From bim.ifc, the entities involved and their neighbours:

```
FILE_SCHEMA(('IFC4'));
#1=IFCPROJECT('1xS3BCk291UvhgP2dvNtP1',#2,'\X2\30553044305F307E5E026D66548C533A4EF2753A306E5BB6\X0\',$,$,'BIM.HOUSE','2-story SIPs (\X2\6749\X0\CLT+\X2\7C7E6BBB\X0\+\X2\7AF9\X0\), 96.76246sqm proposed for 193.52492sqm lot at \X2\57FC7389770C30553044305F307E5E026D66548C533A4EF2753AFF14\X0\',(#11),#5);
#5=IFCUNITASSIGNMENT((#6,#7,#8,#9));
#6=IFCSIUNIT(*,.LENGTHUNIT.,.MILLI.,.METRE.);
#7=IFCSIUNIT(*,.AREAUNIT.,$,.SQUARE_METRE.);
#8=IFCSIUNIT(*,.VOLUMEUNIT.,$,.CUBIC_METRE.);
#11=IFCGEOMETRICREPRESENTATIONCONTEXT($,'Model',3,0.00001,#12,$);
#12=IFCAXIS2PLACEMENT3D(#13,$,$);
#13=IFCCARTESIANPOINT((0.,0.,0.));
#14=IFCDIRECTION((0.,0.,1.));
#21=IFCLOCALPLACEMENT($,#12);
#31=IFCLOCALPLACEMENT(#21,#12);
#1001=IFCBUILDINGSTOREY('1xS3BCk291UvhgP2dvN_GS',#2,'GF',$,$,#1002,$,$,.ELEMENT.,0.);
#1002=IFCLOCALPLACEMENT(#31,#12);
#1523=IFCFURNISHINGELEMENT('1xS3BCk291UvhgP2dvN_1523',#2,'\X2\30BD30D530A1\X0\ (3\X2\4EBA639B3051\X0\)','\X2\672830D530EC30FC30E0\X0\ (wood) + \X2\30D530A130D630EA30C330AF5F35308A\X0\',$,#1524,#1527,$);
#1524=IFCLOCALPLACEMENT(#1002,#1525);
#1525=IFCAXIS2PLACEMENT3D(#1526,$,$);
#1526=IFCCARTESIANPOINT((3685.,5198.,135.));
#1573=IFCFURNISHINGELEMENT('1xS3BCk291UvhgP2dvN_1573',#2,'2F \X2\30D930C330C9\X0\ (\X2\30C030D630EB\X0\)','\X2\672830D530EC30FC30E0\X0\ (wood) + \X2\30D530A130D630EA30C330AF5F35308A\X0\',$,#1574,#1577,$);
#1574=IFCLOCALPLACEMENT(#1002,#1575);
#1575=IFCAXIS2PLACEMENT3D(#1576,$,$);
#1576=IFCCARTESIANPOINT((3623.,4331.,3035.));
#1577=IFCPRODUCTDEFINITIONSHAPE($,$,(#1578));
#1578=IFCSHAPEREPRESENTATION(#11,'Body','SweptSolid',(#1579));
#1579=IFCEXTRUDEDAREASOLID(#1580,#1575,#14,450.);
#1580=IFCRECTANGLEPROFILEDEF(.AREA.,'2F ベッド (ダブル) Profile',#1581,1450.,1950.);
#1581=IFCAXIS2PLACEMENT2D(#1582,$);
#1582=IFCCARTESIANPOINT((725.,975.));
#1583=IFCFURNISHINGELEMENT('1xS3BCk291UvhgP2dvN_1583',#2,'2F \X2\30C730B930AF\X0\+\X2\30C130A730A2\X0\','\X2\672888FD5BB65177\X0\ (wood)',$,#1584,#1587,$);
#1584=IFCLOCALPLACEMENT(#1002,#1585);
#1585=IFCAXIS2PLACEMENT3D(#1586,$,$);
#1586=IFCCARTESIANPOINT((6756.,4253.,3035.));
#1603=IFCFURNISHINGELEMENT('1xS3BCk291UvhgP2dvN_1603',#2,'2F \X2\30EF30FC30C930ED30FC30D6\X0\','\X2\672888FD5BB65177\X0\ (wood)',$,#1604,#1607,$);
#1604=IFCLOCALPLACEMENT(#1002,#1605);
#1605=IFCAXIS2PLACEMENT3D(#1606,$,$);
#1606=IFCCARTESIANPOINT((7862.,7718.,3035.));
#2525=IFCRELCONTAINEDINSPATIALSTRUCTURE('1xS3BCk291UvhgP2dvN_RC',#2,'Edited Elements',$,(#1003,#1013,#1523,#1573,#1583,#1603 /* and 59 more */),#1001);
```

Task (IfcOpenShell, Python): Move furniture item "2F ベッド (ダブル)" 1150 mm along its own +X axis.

```python
import ifcopenshell
import ifcopenshell.api.geometry
import ifcopenshell.util.placement
import ifcopenshell.util.unit

model = ifcopenshell.open("bim.ifc")
unit_scale = ifcopenshell.util.unit.calculate_unit_scale(model)

item = model.by_guid("1xS3BCk291UvhgP2dvN_1573")
matrix = ifcopenshell.util.placement.get_local_placement(item.ObjectPlacement)
matrix[:3, 3] += matrix[:3, 0] * 1.15 / unit_scale
ifcopenshell.api.geometry.edit_object_placement(model, product=item, matrix=matrix, is_si=False)

print(ifcopenshell.util.placement.get_local_placement(item.ObjectPlacement).round(3) + 0.0)

model.write("bim_edited.ifc")
```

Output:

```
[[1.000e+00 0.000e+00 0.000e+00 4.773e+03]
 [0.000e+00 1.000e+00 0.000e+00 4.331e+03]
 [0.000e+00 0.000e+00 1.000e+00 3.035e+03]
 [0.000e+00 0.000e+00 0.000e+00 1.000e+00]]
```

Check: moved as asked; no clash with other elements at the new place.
